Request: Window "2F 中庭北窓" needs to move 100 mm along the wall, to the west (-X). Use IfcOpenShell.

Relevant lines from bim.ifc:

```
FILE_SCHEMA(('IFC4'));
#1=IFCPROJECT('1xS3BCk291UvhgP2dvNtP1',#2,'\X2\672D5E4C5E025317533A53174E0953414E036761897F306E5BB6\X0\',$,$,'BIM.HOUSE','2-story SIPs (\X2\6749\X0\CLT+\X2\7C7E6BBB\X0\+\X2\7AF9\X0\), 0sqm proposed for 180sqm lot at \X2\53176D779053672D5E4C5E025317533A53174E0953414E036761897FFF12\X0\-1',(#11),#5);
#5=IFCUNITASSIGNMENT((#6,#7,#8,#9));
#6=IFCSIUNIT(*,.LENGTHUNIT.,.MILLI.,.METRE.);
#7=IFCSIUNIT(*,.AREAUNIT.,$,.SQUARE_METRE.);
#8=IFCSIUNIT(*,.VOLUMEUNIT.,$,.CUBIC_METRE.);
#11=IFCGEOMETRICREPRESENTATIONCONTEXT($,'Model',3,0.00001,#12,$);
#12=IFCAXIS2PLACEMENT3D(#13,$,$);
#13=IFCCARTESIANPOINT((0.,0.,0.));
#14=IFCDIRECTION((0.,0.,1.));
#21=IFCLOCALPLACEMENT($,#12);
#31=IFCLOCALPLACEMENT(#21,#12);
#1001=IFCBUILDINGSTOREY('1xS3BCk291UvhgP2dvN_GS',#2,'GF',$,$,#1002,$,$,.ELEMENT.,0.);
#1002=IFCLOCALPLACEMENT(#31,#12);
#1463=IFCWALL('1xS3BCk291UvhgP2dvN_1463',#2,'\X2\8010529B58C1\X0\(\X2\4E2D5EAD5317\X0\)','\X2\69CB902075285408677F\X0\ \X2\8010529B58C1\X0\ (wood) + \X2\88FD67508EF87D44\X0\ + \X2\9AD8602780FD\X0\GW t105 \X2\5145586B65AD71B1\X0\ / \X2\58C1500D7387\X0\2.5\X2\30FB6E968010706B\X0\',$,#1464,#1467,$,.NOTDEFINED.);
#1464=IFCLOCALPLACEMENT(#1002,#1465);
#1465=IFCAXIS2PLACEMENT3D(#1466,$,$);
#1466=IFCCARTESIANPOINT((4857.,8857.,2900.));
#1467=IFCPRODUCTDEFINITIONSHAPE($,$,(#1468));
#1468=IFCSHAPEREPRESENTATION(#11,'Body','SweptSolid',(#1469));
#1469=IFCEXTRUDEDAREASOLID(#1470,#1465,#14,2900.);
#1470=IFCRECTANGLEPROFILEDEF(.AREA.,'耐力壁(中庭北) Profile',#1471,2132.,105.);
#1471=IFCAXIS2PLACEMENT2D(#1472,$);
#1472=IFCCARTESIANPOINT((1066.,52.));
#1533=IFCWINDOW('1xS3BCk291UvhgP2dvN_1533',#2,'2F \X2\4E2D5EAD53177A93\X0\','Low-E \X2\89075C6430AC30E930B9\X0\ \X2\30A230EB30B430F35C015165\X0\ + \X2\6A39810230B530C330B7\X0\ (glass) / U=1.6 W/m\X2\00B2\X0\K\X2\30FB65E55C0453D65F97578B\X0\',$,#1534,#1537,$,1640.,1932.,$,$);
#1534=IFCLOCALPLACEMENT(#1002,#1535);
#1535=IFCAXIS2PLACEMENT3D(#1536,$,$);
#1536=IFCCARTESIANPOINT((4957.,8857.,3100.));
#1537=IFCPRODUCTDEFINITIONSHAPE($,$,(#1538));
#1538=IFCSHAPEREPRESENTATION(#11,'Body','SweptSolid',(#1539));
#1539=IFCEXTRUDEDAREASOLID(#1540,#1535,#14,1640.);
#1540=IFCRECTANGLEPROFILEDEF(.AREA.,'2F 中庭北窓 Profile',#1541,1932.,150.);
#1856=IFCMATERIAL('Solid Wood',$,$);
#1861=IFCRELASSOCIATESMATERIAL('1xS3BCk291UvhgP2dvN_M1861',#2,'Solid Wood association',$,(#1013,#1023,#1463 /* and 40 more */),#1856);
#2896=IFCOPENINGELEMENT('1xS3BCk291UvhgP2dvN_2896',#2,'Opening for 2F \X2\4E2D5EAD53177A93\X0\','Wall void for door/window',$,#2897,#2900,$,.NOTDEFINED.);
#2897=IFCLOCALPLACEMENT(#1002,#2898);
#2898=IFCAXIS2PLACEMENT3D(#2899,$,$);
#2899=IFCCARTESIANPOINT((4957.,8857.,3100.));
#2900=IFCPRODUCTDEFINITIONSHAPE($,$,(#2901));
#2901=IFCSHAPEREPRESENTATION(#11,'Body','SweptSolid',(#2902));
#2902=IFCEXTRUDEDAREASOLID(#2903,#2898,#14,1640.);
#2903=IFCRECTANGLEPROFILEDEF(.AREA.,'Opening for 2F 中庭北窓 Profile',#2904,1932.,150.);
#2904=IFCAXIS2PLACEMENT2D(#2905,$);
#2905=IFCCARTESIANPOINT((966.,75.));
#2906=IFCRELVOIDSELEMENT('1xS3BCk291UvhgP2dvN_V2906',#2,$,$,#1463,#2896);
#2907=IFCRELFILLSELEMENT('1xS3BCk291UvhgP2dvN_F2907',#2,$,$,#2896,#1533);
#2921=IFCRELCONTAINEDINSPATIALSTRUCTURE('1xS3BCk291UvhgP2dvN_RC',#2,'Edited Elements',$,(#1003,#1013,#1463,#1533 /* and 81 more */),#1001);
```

```python
import ifcopenshell
import ifcopenshell.api.geometry
import ifcopenshell.util.placement
import ifcopenshell.util.unit

model = ifcopenshell.open("bim.ifc")
unit_scale = ifcopenshell.util.unit.calculate_unit_scale(model)

window = model.by_id(1533)
opening = window.FillsVoids[0].RelatingOpeningElement
wall = opening.VoidsElements[0].RelatingBuildingElement

wall_matrix = ifcopenshell.util.placement.get_local_placement(wall.ObjectPlacement)
shift = wall_matrix[:3, 0] * -0.1 / unit_scale
before = ifcopenshell.util.placement.get_local_placement(window.ObjectPlacement)[:3, 3].copy()

# The window is not placed relative to its opening, so move both.
for product in (opening, window):
    matrix = ifcopenshell.util.placement.get_local_placement(product.ObjectPlacement)
    matrix[:3, 3] += shift
    ifcopenshell.api.geometry.edit_object_placement(model, product=product, matrix=matrix, is_si=False)

after = ifcopenshell.util.placement.get_local_placement(window.ObjectPlacement)[:3, 3]
print("window moved by", (after - before).round(3) + 0.0)

model.write("bim_v2.ifc")
```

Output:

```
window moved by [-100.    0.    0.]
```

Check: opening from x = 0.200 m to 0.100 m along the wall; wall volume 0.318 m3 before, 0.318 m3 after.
